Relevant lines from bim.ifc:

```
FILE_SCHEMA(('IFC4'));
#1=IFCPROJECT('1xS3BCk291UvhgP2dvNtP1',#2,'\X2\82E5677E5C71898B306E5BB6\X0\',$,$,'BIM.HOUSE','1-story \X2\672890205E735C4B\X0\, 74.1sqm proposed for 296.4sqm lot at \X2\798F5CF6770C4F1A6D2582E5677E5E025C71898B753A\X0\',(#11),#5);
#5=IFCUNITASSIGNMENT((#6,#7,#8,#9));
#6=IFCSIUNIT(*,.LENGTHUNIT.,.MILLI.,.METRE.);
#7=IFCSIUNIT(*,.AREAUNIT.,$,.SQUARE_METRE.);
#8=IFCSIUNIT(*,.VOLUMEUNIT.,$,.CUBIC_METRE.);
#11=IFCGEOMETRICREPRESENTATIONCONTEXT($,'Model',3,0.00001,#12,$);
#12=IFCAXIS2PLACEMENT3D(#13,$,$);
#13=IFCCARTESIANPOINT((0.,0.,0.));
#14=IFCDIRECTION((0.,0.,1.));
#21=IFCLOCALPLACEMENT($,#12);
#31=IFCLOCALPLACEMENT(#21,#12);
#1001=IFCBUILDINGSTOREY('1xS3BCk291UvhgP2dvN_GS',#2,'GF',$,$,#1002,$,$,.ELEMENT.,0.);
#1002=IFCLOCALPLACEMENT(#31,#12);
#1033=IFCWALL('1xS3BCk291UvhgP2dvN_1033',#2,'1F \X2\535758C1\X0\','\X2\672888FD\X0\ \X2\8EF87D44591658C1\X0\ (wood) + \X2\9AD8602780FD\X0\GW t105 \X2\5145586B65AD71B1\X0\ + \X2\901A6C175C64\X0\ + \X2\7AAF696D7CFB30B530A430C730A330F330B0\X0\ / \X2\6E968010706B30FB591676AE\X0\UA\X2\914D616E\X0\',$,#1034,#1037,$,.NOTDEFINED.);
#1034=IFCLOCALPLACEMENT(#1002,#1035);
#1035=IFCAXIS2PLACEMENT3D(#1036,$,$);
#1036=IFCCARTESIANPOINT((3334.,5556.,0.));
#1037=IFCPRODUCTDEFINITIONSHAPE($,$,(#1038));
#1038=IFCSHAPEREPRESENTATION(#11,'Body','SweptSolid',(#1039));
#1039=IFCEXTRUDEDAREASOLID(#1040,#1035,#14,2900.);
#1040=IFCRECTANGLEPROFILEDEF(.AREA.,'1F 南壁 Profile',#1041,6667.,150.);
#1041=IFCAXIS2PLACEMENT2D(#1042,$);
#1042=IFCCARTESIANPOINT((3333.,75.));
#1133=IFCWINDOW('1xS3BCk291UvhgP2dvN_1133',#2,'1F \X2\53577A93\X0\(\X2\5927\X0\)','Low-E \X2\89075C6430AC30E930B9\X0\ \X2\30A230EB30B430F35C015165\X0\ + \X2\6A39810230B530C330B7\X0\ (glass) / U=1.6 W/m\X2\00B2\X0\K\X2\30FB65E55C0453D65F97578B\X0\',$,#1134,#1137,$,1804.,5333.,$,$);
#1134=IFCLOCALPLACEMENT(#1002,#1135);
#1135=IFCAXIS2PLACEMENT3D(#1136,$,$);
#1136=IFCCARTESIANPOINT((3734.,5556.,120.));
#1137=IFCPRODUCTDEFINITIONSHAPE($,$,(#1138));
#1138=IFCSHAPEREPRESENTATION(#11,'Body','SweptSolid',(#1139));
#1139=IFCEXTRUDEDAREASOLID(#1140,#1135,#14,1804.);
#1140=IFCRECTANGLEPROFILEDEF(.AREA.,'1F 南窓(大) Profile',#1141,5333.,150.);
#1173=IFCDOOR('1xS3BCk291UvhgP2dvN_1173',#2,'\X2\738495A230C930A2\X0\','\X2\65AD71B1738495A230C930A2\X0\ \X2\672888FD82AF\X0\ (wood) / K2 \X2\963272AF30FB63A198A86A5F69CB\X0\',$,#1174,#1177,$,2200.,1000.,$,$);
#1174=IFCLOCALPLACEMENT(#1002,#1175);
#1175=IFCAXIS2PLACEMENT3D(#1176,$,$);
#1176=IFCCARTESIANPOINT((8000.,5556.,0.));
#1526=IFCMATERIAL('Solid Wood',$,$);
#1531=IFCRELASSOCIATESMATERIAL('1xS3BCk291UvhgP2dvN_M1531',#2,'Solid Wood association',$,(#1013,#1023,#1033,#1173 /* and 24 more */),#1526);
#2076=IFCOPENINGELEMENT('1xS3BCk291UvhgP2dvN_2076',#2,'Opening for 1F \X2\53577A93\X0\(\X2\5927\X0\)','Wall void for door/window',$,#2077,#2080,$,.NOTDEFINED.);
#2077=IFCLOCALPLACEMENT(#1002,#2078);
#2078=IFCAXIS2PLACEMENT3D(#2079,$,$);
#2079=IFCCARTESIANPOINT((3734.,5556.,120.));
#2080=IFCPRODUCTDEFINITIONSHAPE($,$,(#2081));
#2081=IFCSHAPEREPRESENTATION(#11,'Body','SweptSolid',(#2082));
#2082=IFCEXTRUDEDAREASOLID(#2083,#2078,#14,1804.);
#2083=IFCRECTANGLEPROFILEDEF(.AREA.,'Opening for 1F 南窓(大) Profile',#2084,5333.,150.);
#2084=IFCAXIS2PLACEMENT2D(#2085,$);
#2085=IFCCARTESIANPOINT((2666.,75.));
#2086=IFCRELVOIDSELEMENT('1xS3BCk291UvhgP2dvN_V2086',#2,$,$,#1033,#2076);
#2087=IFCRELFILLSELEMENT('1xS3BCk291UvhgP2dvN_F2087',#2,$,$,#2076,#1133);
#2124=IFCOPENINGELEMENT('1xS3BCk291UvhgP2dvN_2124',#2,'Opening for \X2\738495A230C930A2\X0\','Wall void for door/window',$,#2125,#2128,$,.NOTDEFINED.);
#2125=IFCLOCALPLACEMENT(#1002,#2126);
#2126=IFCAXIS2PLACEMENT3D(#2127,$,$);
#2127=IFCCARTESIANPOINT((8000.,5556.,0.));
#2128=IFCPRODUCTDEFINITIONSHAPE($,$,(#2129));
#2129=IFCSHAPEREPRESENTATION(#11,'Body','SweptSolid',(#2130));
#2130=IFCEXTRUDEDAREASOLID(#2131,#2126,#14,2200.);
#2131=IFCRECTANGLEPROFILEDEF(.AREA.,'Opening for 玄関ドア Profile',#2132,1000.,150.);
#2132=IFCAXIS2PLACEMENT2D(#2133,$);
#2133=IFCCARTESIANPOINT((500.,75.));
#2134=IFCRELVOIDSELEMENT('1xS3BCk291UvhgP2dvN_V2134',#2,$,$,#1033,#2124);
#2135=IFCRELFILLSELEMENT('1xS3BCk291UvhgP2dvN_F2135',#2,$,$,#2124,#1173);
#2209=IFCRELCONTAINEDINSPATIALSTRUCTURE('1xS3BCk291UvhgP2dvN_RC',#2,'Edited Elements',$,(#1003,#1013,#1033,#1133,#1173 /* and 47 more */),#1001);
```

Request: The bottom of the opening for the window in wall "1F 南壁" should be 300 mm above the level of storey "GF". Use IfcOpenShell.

```python
import numpy as np
import ifcopenshell
import ifcopenshell.api.geometry
import ifcopenshell.geom
import ifcopenshell.util.element
import ifcopenshell.util.placement
import ifcopenshell.util.shape
import ifcopenshell.util.unit

model = ifcopenshell.open("bim.ifc")
unit_scale = ifcopenshell.util.unit.calculate_unit_scale(model)

window = model.by_id(1133)
opening = window.FillsVoids[0].RelatingOpeningElement
storey = ifcopenshell.util.element.get_container(window, ifc_class="IfcBuildingStorey")
level = ifcopenshell.util.placement.get_local_placement(storey.ObjectPlacement)[2, 3]

# The opening's origin need not be at the sill, so measure its lowest point.
shape = ifcopenshell.geom.create_shape(ifcopenshell.geom.settings(), opening)
bottom = ifcopenshell.util.shape.get_shape_bottom_elevation(shape, shape.geometry) / unit_scale
dz = level + 0.3 / unit_scale - bottom

shift = np.array([0.0, 0.0, dz])
# The window is not placed relative to its opening, so move both.
for product in (opening, window):
    matrix = ifcopenshell.util.placement.get_local_placement(product.ObjectPlacement)
    matrix[:3, 3] += shift
    ifcopenshell.api.geometry.edit_object_placement(model, product=product, matrix=matrix, is_si=False)

print(f"moved by {dz * unit_scale:+.3f} m")

model.write("bim_rev.ifc")
```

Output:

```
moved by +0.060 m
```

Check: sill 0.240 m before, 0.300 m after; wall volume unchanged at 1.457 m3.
